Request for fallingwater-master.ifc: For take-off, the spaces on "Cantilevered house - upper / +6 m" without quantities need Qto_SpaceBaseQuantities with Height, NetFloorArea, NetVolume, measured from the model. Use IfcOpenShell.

First a look at what the model holds.

```python
import ifcopenshell
import ifcopenshell.util.element
import ifcopenshell.util.unit

model = ifcopenshell.open("fallingwater-master.ifc")
print(model.schema)
for unit_type in ("LENGTHUNIT", "AREAUNIT", "VOLUMEUNIT"):
    print(unit_type, ifcopenshell.util.unit.calculate_unit_scale(model, unit_type))
storey = next(s for s in model.by_type("IfcBuildingStorey") if s.Name == "Cantilevered house - upper / +6 m")
spaces = [e for e in ifcopenshell.util.element.get_decomposition(storey) if e.is_a("IfcSpace")]
for e in sorted(spaces, key=lambda e: e.id()):
    print(e.id(), e.is_a(), e.Name, list(ifcopenshell.util.element.get_psets(e, qtos_only=True)), sep=" | ")
```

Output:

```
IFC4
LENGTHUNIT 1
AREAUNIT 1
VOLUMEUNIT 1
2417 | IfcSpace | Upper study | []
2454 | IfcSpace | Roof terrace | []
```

```python
import ifcopenshell
import ifcopenshell.api.pset
import ifcopenshell.geom
import ifcopenshell.util.element
import ifcopenshell.util.shape
import ifcopenshell.util.unit

model = ifcopenshell.open("fallingwater-master.ifc")
unit_scale = ifcopenshell.util.unit.calculate_unit_scale(model)
area_scale = ifcopenshell.util.unit.calculate_unit_scale(model, "AREAUNIT")
volume_scale = ifcopenshell.util.unit.calculate_unit_scale(model, "VOLUMEUNIT")
settings = ifcopenshell.geom.settings()

storey = next(s for s in model.by_type("IfcBuildingStorey") if s.Name == "Cantilevered house - upper / +6 m")
spaces = [e for e in ifcopenshell.util.element.get_decomposition(storey) if e.is_a("IfcSpace")]

for e in sorted(spaces, key=lambda e: e.id()):
    if ifcopenshell.util.element.get_psets(e, qtos_only=True, should_inherit=False):
        continue
    # Geometry comes back in metres, in the element's own axes.
    shape = ifcopenshell.geom.create_shape(settings, e)
    values = {
        "Height": ifcopenshell.util.shape.get_z(shape.geometry) / unit_scale,
        "NetFloorArea": ifcopenshell.util.shape.get_footprint_area(shape.geometry) / area_scale,
        "NetVolume": ifcopenshell.util.shape.get_volume(shape.geometry) / volume_scale,
    }
    qto = ifcopenshell.api.pset.add_qto(model, product=e, name="Qto_SpaceBaseQuantities")
    ifcopenshell.api.pset.edit_qto(model, qto=qto, properties=values)
    print(e.id(), {k: round(v, 3) for k, v in values.items()})

model.write("fallingwater-master-out.ifc")
```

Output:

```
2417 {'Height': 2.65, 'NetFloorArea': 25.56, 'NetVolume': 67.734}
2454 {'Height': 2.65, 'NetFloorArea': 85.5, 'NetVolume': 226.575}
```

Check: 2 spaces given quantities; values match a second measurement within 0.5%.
